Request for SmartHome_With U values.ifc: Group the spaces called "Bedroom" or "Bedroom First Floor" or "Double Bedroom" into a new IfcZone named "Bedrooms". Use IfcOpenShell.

First a look at what the model holds.

```python
import ifcopenshell

model = ifcopenshell.open("SmartHome_With U values.ifc")
print(model.schema)
seen = {}
for space in model.by_type("IfcSpace"):
    seen[space.LongName] = seen.get(space.LongName, 0) + 1
for name, count in sorted(seen.items(), key=str):
    print(count, "x", name)
print("zones:", [z.Name for z in model.by_type("IfcZone")][:20])
```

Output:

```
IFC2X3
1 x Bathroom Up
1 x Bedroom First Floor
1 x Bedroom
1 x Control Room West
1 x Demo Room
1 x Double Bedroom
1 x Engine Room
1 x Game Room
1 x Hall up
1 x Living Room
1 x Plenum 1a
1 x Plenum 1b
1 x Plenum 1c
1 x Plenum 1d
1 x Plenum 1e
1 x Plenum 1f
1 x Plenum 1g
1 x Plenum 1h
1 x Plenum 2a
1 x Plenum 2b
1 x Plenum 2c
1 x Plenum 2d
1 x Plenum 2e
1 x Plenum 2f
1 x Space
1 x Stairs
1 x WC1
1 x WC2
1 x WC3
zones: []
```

```python
import ifcopenshell
import ifcopenshell.api.group
import ifcopenshell.api.root

model = ifcopenshell.open("SmartHome_With U values.ifc")

names = {"Bedroom", "Bedroom First Floor", "Double Bedroom"}
spaces = [s for s in model.by_type("IfcSpace") if s.LongName in names]

zone = ifcopenshell.api.root.create_entity(model, ifc_class="IfcZone", name="Bedrooms")
ifcopenshell.api.group.assign_group(model, products=spaces, group=zone)
print(len(spaces), "spaces in", zone.Name)

model.write("SmartHome_With U values_v2.ifc")
```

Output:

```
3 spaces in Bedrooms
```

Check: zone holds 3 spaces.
